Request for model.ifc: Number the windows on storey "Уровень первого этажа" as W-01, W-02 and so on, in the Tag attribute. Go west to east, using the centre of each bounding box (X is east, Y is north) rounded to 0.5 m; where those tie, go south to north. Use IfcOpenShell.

First a look at what the model holds.

```python
import ifcopenshell
import ifcopenshell.util.element
import ifcopenshell.util.placement

model = ifcopenshell.open("model.ifc")
print(model.schema)
storey = next(s for s in model.by_type("IfcBuildingStorey") if s.Name == "Уровень первого этажа")
windows = [e for e in ifcopenshell.util.element.get_decomposition(storey) if e.is_a("IfcWindow")]
for e in sorted(windows, key=lambda e: e.id()):
    origin = ifcopenshell.util.placement.get_local_placement(e.ObjectPlacement)[:3, 3]
    print(e.id(), e.Tag, e.Name, origin.round(2) + 0.0, sep=" | ")
```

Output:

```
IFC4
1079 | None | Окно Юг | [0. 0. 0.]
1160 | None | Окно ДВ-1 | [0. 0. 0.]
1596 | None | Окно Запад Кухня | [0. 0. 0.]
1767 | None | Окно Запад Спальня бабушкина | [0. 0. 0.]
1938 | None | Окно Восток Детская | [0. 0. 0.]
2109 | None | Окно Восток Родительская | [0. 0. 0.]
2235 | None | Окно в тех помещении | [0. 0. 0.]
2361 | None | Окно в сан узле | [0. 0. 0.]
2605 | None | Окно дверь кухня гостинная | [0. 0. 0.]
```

```python
import ifcopenshell
import ifcopenshell.geom
import ifcopenshell.util.element
import ifcopenshell.util.shape

model = ifcopenshell.open("model.ifc")
settings = ifcopenshell.geom.settings()
settings.set("use-world-coords", True)


def centre(element):
    shape = ifcopenshell.geom.create_shape(settings, element)
    return ifcopenshell.util.shape.get_bbox_centroid(shape.geometry)


storey = next(s for s in model.by_type("IfcBuildingStorey") if s.Name == "Уровень первого этажа")
windows = [e for e in ifcopenshell.util.element.get_decomposition(storey) if e.is_a("IfcWindow")]

# Insertion points can sit at a corner or the storey origin, so sort by the geometry (in metres).
centres = {e: centre(e) for e in windows}
windows.sort(key=lambda e: (round(centres[e][0] / 0.5), centres[e][1]))

for i, e in enumerate(windows, start=1):
    number = f"W-{i:02d}"
    e.Tag = number
    print(e.id(), number)

model.write("model_v2.ifc")
```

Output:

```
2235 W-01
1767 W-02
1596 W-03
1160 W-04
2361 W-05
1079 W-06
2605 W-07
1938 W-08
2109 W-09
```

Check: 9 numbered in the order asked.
